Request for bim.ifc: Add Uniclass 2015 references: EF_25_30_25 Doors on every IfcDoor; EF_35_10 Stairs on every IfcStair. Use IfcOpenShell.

First a look at what the model holds.

```python
import ifcopenshell

model = ifcopenshell.open("bim.ifc")
print(model.schema)
print("classifications:", [c.Name for c in model.by_type("IfcClassification")])
for ifc_class in ("IfcDoor", "IfcRoof", "IfcStair", "IfcWall", "IfcWindow"):
    print(ifc_class, len(model.by_type(ifc_class)))
```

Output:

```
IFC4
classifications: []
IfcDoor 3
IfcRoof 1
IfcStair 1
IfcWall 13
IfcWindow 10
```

```python
import ifcopenshell
import ifcopenshell.api.classification

model = ifcopenshell.open("bim.ifc")

system = ifcopenshell.api.classification.add_classification(model, classification="Uniclass 2015")

codes = {
    "IfcDoor": ("EF_25_30_25", "Doors"),
    "IfcStair": ("EF_35_10", "Stairs"),
}
for ifc_class, (code, name) in codes.items():
    products = model.by_type(ifc_class)
    ifcopenshell.api.classification.add_reference(
        model, products=products, classification=system, identification=code, name=name
    )
    print(code, len(products))

model.write("bim_updated.ifc")
```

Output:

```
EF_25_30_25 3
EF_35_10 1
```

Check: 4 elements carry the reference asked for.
